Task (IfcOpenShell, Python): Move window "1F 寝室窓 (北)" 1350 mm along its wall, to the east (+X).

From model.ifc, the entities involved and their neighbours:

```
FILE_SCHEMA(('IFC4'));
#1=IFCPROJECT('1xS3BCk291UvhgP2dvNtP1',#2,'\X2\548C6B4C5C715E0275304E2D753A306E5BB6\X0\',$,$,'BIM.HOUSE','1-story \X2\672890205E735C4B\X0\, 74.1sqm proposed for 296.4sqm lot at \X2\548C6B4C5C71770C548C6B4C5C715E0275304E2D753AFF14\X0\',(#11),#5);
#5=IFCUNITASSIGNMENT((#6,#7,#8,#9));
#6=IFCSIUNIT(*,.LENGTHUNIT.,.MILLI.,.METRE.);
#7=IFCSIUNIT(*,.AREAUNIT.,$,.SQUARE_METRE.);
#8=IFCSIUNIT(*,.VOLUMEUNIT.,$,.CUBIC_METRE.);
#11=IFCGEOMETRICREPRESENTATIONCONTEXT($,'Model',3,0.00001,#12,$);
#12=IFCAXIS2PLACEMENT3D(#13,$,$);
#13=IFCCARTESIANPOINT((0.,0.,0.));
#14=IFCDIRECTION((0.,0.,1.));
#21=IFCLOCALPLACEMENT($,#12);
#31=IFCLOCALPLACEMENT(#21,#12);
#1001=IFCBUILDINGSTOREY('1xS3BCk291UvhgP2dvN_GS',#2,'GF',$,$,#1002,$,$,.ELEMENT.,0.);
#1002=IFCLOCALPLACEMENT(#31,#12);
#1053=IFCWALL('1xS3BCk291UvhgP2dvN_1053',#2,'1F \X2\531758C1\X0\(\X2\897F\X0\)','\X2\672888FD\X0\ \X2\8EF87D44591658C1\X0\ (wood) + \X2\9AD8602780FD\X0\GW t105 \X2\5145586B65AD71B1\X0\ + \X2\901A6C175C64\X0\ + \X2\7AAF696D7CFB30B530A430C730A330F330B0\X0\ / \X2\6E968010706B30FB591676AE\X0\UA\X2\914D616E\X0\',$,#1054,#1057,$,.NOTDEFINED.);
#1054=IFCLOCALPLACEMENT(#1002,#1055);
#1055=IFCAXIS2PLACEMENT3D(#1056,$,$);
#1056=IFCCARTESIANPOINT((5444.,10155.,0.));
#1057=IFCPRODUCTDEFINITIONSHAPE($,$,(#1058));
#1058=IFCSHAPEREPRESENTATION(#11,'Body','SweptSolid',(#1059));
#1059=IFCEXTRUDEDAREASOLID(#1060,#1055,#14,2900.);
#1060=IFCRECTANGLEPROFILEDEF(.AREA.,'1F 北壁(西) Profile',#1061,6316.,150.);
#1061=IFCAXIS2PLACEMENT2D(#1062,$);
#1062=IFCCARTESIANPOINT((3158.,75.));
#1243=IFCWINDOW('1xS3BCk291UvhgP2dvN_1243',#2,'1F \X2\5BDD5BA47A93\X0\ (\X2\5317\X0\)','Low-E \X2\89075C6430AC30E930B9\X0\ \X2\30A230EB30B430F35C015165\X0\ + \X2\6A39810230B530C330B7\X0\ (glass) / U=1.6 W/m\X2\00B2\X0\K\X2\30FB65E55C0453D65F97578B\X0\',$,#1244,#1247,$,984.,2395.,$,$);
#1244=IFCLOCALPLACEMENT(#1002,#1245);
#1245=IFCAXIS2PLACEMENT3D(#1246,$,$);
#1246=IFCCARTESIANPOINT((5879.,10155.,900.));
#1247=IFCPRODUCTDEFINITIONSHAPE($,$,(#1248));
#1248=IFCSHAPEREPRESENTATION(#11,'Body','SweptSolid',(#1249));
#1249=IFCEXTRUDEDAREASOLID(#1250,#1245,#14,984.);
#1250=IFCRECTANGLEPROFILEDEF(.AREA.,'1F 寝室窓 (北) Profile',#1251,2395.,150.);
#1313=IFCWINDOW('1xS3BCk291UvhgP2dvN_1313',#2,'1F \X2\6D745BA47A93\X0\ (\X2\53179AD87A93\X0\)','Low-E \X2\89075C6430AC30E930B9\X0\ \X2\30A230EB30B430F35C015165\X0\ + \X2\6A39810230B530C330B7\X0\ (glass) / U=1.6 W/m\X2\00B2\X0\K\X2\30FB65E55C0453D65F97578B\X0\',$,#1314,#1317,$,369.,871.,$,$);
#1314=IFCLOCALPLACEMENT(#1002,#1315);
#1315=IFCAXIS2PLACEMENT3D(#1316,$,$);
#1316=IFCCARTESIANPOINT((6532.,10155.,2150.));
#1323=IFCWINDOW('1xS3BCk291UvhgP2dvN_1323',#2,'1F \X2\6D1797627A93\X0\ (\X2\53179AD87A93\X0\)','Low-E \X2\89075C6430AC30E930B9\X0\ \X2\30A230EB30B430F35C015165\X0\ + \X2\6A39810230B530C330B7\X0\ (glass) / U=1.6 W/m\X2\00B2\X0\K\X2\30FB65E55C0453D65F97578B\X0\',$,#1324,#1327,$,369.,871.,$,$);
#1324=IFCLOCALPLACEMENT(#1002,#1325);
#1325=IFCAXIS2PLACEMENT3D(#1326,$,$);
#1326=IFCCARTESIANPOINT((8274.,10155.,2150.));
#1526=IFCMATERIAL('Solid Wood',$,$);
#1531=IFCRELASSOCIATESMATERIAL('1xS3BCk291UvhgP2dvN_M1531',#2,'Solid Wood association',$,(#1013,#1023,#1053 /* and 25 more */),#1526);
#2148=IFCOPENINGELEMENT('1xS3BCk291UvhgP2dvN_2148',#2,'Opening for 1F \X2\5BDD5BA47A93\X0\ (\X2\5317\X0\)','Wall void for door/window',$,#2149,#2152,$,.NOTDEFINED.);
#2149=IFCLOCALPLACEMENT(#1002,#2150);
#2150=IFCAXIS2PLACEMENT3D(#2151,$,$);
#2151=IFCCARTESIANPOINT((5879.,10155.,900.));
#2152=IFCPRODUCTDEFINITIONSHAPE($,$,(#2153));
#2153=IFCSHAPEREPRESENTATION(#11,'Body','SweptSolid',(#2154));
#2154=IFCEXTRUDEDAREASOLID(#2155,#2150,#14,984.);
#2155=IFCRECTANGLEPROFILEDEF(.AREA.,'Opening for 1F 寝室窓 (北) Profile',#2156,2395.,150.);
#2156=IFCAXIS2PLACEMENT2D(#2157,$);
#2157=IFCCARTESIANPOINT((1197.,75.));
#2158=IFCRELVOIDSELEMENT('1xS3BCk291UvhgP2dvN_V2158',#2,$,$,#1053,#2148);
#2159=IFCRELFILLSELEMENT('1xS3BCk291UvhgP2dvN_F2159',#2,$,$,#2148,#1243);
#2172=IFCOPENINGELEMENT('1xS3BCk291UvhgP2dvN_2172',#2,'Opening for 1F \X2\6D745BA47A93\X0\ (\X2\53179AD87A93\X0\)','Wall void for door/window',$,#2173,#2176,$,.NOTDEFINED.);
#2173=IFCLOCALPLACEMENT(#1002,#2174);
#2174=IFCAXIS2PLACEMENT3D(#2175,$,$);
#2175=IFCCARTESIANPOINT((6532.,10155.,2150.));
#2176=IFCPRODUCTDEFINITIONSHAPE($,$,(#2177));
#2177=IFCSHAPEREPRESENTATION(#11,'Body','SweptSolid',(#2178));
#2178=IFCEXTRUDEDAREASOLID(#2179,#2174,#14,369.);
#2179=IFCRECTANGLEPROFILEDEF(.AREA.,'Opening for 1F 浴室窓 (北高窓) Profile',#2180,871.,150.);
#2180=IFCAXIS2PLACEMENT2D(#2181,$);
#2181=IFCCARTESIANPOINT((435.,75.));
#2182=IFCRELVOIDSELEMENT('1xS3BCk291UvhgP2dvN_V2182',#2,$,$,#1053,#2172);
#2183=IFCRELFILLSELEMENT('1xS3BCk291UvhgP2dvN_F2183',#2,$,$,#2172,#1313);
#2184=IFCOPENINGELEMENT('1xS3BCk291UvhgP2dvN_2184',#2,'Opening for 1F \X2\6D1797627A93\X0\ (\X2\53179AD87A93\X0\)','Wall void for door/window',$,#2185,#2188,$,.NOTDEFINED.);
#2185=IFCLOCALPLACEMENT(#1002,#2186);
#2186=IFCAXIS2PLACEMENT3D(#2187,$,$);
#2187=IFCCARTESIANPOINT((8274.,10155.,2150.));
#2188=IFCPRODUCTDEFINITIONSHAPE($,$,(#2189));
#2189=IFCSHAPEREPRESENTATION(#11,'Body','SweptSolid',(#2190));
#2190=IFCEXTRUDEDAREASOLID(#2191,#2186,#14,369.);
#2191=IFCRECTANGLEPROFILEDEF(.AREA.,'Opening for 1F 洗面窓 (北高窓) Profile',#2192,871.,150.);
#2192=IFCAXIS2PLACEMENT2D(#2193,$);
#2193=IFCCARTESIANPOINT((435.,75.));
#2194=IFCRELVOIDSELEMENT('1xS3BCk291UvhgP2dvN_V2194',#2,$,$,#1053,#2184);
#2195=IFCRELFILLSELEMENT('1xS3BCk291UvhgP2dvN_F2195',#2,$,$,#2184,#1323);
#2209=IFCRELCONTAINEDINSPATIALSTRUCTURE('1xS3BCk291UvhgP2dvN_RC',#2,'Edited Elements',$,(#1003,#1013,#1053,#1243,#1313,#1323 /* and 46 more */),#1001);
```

```python
import ifcopenshell
import ifcopenshell.api.geometry
import ifcopenshell.util.placement
import ifcopenshell.util.unit

model = ifcopenshell.open("model.ifc")
unit_scale = ifcopenshell.util.unit.calculate_unit_scale(model)

window = model.by_id(1243)
opening = window.FillsVoids[0].RelatingOpeningElement
wall = opening.VoidsElements[0].RelatingBuildingElement

wall_matrix = ifcopenshell.util.placement.get_local_placement(wall.ObjectPlacement)
shift = wall_matrix[:3, 0] * 1.35 / unit_scale
before = ifcopenshell.util.placement.get_local_placement(window.ObjectPlacement)[:3, 3].copy()

# The window is not placed relative to its opening, so move both.
for product in (opening, window):
    matrix = ifcopenshell.util.placement.get_local_placement(product.ObjectPlacement)
    matrix[:3, 3] += shift
    ifcopenshell.api.geometry.edit_object_placement(model, product=product, matrix=matrix, is_si=False)

after = ifcopenshell.util.placement.get_local_placement(window.ObjectPlacement)[:3, 3]
print("window moved by", (after - before).round(3) + 0.0)

model.write("model_edited.ifc")
```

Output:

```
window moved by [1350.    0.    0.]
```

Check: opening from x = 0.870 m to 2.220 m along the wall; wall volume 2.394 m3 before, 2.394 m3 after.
